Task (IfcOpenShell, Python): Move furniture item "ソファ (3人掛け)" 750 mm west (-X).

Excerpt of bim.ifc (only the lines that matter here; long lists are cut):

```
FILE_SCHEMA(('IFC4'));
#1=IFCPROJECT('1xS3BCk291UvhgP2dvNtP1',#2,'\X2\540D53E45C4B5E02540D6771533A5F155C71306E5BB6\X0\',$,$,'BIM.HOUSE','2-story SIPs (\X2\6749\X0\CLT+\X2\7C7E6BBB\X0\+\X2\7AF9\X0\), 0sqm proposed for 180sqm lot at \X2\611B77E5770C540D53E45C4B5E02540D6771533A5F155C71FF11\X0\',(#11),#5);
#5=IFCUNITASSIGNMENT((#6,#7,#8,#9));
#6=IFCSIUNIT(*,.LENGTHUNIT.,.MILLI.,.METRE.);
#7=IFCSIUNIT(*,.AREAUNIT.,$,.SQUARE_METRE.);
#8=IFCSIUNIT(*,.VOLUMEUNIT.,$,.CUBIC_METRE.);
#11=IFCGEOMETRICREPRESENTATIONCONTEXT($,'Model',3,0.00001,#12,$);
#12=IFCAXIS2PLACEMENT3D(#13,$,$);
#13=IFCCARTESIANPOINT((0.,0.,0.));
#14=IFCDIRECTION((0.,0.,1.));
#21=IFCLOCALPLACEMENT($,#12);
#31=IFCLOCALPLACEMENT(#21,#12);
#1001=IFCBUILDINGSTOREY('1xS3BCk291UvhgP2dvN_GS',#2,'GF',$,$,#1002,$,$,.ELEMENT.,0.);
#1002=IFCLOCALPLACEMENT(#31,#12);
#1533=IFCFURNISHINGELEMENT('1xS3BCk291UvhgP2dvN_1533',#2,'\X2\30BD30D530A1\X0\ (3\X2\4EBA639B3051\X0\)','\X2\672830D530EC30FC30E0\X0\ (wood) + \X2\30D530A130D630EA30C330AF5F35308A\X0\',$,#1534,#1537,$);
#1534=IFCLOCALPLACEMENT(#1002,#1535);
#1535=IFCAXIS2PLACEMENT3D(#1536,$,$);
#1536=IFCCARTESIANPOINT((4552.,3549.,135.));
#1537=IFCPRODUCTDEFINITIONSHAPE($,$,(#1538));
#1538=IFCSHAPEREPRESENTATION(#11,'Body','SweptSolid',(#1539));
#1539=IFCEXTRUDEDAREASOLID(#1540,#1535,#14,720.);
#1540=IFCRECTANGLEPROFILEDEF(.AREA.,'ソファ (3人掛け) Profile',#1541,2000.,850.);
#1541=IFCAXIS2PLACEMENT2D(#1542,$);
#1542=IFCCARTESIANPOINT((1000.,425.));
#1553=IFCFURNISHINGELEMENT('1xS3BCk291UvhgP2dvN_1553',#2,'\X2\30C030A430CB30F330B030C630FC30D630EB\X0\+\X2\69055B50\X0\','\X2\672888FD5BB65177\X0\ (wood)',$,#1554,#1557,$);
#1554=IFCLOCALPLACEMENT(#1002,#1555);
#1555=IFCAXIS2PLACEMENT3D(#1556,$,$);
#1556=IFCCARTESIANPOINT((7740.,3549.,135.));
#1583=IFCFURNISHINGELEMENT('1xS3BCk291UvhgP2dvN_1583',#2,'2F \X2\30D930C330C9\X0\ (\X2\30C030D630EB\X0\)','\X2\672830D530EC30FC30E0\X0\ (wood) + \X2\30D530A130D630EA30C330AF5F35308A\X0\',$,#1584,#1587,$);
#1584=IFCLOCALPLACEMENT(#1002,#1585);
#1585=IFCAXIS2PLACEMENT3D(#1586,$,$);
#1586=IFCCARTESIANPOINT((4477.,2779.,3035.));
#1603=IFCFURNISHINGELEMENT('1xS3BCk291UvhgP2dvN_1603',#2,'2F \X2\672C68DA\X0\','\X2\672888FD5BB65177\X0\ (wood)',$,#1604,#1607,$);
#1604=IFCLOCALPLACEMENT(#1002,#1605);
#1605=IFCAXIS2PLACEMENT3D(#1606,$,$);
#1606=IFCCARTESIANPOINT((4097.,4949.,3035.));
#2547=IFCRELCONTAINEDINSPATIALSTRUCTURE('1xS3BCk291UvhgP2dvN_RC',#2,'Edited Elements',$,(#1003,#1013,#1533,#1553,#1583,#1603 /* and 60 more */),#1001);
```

```python
import ifcopenshell
import ifcopenshell.api.geometry
import ifcopenshell.util.placement

model = ifcopenshell.open("bim.ifc")

item = model.by_id(1533)
matrix = ifcopenshell.util.placement.get_local_placement(item.ObjectPlacement)
matrix[0, 3] -= 750.0
ifcopenshell.api.geometry.edit_object_placement(model, product=item, matrix=matrix, is_si=False)

print(ifcopenshell.util.placement.get_local_placement(item.ObjectPlacement).round(3) + 0.0)

model.write("bim_rev.ifc")
```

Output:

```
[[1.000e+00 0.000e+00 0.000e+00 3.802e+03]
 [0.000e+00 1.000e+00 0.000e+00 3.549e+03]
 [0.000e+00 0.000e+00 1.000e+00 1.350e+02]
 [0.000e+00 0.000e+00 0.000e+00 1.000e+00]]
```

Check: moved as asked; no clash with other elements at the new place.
